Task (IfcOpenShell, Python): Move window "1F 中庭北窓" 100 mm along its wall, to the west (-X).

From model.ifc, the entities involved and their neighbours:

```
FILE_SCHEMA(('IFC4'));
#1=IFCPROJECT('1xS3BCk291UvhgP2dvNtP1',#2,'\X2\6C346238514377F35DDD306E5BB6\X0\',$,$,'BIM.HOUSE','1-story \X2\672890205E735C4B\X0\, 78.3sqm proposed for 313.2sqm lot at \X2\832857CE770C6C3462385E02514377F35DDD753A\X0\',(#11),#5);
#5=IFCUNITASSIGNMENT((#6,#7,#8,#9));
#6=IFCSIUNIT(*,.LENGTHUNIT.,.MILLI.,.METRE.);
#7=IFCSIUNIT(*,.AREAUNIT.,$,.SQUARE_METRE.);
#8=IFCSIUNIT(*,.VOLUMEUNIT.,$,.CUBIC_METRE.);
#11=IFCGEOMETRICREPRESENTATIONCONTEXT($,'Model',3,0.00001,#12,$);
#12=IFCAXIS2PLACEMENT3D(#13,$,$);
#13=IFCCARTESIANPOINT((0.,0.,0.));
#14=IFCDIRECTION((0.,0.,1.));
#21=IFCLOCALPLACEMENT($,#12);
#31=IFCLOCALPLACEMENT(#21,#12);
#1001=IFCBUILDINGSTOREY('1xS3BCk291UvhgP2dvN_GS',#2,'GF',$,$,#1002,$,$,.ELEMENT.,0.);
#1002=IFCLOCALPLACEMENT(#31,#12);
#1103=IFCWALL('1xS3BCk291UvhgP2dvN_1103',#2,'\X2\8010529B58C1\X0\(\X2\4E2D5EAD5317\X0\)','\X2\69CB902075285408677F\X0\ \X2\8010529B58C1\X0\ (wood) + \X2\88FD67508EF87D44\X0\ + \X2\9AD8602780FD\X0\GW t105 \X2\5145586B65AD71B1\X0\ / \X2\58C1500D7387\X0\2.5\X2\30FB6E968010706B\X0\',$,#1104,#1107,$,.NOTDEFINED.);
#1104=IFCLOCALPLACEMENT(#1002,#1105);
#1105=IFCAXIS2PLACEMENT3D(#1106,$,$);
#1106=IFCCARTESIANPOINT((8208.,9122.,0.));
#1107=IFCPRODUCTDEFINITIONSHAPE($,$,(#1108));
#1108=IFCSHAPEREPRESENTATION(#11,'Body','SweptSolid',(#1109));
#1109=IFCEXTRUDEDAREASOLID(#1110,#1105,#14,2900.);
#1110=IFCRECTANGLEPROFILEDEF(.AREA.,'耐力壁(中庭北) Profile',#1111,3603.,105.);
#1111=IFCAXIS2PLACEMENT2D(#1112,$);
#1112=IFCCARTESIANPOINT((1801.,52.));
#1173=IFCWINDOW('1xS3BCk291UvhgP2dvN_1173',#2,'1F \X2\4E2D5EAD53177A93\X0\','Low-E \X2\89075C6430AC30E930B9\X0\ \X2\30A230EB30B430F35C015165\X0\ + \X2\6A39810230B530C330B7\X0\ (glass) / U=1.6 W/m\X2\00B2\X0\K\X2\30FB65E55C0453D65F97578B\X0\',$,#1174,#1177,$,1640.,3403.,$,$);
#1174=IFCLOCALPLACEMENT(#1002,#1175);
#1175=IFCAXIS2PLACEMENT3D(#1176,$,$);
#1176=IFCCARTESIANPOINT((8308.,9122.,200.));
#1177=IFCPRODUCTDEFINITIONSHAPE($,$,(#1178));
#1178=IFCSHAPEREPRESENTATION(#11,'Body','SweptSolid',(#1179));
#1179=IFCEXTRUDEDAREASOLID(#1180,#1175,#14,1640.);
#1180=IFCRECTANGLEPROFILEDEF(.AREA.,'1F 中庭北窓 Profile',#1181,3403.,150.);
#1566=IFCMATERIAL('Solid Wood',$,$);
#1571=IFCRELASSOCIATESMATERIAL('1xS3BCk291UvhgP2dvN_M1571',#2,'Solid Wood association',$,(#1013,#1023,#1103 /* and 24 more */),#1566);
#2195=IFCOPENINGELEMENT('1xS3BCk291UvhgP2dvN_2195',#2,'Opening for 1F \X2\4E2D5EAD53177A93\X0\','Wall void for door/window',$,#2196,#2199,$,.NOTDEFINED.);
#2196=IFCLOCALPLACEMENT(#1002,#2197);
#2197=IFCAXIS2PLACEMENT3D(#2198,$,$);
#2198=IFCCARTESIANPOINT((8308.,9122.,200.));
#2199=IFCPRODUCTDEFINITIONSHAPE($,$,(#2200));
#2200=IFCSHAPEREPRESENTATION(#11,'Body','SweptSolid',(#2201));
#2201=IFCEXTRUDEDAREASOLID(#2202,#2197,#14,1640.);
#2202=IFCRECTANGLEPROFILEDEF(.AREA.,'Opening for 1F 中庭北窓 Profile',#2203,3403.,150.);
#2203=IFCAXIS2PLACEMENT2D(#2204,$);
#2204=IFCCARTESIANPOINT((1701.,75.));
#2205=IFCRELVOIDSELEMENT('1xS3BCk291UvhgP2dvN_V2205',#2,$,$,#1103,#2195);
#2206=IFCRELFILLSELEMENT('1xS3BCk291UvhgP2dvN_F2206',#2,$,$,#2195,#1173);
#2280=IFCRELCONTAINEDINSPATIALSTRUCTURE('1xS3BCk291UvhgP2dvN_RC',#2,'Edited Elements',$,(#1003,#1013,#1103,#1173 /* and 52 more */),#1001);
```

```python
import ifcopenshell
import ifcopenshell.api.geometry
import ifcopenshell.util.placement

model = ifcopenshell.open("model.ifc")

window = model.by_guid("1xS3BCk291UvhgP2dvN_1173")
opening = window.FillsVoids[0].RelatingOpeningElement
wall = opening.VoidsElements[0].RelatingBuildingElement

wall_matrix = ifcopenshell.util.placement.get_local_placement(wall.ObjectPlacement)
shift = wall_matrix[:3, 0] * -100.0
before = ifcopenshell.util.placement.get_local_placement(window.ObjectPlacement)[:3, 3].copy()

# The window is not placed relative to its opening, so move both.
for product in (opening, window):
    matrix = ifcopenshell.util.placement.get_local_placement(product.ObjectPlacement)
    matrix[:3, 3] += shift
    ifcopenshell.api.geometry.edit_object_placement(model, product=product, matrix=matrix, is_si=False)

after = ifcopenshell.util.placement.get_local_placement(window.ObjectPlacement)[:3, 3]
print("window moved by", (after - before).round(3) + 0.0)

model.write("model_v2.ifc")
```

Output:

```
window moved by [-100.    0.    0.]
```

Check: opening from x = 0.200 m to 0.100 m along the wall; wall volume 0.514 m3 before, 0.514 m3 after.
